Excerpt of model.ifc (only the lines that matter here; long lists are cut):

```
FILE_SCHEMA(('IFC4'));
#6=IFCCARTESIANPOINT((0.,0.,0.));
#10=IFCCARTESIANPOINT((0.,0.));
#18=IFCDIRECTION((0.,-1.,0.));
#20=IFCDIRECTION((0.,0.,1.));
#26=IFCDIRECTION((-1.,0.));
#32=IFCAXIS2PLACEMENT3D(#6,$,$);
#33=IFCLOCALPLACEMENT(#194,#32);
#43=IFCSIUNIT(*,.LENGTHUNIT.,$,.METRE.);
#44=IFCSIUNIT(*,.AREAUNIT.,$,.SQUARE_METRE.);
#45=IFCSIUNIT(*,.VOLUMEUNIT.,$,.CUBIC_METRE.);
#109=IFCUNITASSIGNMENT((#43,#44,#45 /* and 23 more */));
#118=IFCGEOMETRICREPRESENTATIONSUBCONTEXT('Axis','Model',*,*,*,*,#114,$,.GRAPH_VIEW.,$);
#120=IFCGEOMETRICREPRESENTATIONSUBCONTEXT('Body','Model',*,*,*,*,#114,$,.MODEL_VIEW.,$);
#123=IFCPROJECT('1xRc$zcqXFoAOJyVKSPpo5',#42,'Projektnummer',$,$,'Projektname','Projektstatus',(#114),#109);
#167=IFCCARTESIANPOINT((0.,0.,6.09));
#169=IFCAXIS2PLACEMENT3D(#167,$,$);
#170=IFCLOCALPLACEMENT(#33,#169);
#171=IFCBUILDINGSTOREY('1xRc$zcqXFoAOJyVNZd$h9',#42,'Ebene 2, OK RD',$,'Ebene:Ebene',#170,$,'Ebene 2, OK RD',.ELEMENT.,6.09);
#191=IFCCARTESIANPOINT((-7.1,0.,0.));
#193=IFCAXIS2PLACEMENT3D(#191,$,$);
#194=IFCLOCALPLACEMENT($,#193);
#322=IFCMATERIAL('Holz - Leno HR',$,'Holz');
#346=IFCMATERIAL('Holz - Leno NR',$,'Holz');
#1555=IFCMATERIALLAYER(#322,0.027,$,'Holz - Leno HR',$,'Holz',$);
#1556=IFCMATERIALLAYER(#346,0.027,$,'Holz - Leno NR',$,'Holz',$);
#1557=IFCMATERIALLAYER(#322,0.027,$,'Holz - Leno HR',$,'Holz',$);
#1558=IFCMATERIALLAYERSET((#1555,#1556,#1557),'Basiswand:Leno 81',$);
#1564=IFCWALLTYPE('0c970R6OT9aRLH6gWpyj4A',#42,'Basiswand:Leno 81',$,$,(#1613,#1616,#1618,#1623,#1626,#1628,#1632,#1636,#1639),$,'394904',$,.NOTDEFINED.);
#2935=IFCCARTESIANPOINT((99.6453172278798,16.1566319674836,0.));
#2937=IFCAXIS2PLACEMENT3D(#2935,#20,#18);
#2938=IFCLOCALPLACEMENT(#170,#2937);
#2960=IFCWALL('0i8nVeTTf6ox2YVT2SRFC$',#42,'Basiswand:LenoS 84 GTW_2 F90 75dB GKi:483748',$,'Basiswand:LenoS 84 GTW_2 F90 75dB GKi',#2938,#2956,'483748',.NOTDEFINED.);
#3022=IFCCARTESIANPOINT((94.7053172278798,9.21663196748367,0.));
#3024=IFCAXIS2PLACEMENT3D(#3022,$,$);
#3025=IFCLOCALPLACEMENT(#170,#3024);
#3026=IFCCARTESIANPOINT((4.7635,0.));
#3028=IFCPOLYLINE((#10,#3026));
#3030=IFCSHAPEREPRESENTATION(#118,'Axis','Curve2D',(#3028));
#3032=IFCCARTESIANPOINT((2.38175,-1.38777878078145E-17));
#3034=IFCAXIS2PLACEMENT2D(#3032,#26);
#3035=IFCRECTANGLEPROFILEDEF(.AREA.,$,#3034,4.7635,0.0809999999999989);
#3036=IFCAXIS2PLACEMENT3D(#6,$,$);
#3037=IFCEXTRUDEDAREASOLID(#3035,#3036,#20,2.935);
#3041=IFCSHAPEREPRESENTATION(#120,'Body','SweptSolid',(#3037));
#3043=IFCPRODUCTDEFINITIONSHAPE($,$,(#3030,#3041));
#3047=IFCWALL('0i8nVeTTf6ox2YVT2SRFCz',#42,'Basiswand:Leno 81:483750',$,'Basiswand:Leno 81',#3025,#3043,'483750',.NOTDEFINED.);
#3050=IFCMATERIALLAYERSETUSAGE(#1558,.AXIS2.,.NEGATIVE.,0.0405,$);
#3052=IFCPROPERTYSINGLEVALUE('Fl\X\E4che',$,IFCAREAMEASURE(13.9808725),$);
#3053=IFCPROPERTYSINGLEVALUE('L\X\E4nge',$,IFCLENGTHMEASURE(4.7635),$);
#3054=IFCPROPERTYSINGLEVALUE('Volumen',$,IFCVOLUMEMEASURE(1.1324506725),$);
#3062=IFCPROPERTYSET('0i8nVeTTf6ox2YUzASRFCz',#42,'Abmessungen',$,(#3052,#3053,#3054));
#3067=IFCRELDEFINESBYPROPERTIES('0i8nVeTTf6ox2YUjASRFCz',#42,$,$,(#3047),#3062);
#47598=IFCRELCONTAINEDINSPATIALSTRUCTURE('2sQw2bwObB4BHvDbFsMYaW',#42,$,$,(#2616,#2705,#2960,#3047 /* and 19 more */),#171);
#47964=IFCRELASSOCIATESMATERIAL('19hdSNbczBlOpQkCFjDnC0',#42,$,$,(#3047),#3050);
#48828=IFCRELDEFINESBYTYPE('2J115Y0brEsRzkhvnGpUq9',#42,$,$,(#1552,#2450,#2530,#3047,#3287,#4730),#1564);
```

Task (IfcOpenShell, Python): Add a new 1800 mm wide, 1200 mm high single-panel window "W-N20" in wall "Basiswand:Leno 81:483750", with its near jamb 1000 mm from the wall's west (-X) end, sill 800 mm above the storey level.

```python
import numpy as np
import ifcopenshell
import ifcopenshell.api.feature
import ifcopenshell.api.geometry
import ifcopenshell.api.pset
import ifcopenshell.api.root
import ifcopenshell.api.spatial
import ifcopenshell.geom
import ifcopenshell.util.element
import ifcopenshell.util.placement
import ifcopenshell.util.representation
import ifcopenshell.util.shape
import ifcopenshell.util.unit

model = ifcopenshell.open("model.ifc")
unit_scale = ifcopenshell.util.unit.calculate_unit_scale(model)
area_scale = ifcopenshell.util.unit.calculate_unit_scale(model, "AREAUNIT")
volume_scale = ifcopenshell.util.unit.calculate_unit_scale(model, "VOLUMEUNIT")
settings = ifcopenshell.geom.settings()


def volume(element):
    """Net volume in cubic metres, openings subtracted."""
    shape = ifcopenshell.geom.create_shape(settings, element)
    return ifcopenshell.util.shape.get_volume(shape.geometry)


wall = model.by_guid("0i8nVeTTf6ox2YVT2SRFCz")
storey = ifcopenshell.util.element.get_container(wall, ifc_class="IfcBuildingStorey")
context = ifcopenshell.util.representation.get_context(model, "Model", "Body", "MODEL_VIEW")
before = volume(wall)

width, height, from_end, sill = 1.8, 1.2, 1, 0.8  # metres

# The wall runs along its own X axis, and the end named is its -X end.
wall_shape = ifcopenshell.geom.create_shape(settings, wall)
x, y, z = ifcopenshell.util.shape.get_vertices(wall_shape.geometry).T
start = x.min() + from_end
face, thickness = float(y.min()), float(y.max() - y.min())
wall_matrix = ifcopenshell.util.placement.get_local_placement(wall.ObjectPlacement)
level = ifcopenshell.util.placement.get_local_placement(storey.ObjectPlacement)[2, 3]


def in_wall(x, y):
    """Placement at x, y metres in the wall's axes, at sill height."""
    matrix = wall_matrix.copy()
    matrix[:, 3] = wall_matrix @ np.array([x / unit_scale, y / unit_scale, 0.0, 1.0])
    matrix[2, 3] = level + sill / unit_scale
    return matrix


# Opening: a box that overshoots both wall faces by 50 mm.
opening = ifcopenshell.api.root.create_entity(model, ifc_class="IfcOpeningElement", predefined_type="OPENING")
box = ifcopenshell.api.geometry.add_wall_representation(
    model, context=context, length=width, height=height, thickness=thickness + 0.1
)
ifcopenshell.api.geometry.assign_representation(model, product=opening, representation=box)
ifcopenshell.api.geometry.edit_object_placement(model, product=opening, matrix=in_wall(start, face - 0.05), is_si=False)
ifcopenshell.api.feature.add_feature(model, feature=opening, element=wall)

window = ifcopenshell.api.root.create_entity(model, ifc_class="IfcWindow", name="W-N20", predefined_type="WINDOW")
window.OverallWidth, window.OverallHeight = width / unit_scale, height / unit_scale
window.PartitioningType = "SINGLE_PANEL"
body = ifcopenshell.api.geometry.add_window_representation(
    model,
    context=context,
    overall_width=window.OverallWidth,
    overall_height=window.OverallHeight,
    partition_type="SINGLE_PANEL",
)
ifcopenshell.api.geometry.assign_representation(model, product=window, representation=body)
ifcopenshell.api.spatial.assign_container(model, products=[window], relating_structure=storey)
ifcopenshell.api.feature.add_filling(model, opening=opening, element=window)

# Centre the window in the wall's thickness.
ifcopenshell.api.geometry.edit_object_placement(model, product=window, matrix=in_wall(start, face), is_si=False)
window_shape = ifcopenshell.geom.create_shape(settings, window)
depth = ifcopenshell.util.shape.get_vertices(window_shape.geometry)[:, 1]
offset = face + thickness / 2 - (depth.min() + depth.max()) / 2
ifcopenshell.api.geometry.edit_object_placement(model, product=window, matrix=in_wall(start, offset), is_si=False)

after = volume(wall)

# Update the wall's stored quantities.
pset = model.by_id(ifcopenshell.util.element.get_pset(wall, "Abmessungen", should_inherit=False)["id"])
ifcopenshell.api.pset.edit_pset(model, pset=pset, properties={
    "Fläche": model.create_entity("IfcAreaMeasure", after / thickness / area_scale),
    "Volumen": model.create_entity("IfcVolumeMeasure", after / volume_scale),
})

print(f"wall volume {before:.3f} -> {after:.3f} m3")

model.write("model_updated.ifc")
```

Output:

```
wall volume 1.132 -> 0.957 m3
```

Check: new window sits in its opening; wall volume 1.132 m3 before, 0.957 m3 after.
